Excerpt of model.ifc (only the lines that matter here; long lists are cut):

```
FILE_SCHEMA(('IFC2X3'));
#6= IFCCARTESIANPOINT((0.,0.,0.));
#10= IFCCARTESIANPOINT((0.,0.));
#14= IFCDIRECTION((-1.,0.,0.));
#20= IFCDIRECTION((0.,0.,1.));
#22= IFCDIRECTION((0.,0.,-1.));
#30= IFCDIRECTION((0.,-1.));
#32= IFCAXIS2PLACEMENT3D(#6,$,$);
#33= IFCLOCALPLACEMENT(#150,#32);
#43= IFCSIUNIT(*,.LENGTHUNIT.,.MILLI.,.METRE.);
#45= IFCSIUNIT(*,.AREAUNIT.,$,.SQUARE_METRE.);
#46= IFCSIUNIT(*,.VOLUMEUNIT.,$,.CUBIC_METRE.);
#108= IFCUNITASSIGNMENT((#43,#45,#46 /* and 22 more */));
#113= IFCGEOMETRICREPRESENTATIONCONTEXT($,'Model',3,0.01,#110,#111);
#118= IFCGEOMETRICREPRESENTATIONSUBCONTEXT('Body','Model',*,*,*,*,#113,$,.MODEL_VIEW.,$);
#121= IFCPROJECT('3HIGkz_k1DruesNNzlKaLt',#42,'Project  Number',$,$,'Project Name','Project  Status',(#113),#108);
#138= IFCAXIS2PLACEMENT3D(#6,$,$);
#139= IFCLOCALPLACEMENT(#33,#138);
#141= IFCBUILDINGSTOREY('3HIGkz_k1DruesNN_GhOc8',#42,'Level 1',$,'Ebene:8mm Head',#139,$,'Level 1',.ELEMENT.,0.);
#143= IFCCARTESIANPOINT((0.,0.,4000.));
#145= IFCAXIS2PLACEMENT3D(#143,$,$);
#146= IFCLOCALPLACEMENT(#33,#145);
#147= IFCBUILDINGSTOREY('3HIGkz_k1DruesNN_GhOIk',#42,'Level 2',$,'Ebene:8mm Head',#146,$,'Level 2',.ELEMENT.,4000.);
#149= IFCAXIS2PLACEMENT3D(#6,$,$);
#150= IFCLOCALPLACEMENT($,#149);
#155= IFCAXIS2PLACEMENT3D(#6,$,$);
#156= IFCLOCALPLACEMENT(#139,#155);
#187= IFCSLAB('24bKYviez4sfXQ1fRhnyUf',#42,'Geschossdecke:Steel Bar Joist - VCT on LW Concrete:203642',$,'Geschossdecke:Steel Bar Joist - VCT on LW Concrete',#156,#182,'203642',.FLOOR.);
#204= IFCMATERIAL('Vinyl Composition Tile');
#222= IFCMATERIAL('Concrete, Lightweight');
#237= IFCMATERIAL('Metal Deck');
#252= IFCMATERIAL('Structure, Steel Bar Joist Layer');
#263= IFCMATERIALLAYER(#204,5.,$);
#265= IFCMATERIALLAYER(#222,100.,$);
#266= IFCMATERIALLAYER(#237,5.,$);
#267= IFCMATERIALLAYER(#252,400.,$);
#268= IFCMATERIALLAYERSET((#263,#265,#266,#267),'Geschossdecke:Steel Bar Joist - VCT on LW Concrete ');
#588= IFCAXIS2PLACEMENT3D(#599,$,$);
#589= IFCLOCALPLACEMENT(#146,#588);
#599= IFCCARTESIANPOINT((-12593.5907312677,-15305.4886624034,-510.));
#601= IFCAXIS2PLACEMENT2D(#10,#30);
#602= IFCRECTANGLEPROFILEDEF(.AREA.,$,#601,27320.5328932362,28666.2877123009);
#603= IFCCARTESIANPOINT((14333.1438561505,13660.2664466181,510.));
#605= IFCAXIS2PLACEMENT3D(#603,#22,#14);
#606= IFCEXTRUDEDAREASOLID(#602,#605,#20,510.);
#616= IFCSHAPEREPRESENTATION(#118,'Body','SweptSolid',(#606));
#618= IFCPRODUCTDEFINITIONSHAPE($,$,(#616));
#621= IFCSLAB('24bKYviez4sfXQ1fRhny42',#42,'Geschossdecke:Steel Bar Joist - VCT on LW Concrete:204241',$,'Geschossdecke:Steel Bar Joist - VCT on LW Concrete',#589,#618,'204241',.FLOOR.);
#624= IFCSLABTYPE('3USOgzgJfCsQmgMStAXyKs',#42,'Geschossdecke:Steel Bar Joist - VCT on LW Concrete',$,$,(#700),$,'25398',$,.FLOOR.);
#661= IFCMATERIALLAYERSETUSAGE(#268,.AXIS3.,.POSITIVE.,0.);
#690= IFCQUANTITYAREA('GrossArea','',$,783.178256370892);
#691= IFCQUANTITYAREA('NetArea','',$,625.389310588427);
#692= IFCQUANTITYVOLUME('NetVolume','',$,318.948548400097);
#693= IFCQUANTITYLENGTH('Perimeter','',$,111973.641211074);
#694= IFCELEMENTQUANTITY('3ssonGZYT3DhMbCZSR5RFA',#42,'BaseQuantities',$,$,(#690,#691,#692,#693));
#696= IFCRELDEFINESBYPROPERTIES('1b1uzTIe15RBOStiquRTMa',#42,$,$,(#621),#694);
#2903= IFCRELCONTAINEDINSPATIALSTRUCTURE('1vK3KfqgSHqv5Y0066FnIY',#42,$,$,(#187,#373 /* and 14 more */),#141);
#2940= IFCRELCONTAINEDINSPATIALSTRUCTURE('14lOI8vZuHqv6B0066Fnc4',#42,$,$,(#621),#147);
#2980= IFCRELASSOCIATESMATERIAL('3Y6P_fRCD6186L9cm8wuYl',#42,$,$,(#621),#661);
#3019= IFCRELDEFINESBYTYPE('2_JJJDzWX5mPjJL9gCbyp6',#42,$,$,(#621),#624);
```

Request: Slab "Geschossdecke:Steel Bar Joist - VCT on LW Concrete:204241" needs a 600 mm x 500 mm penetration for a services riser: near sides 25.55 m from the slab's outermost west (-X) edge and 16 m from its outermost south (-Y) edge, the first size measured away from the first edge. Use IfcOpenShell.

```python
import numpy as np
import ifcopenshell
import ifcopenshell.api.feature
import ifcopenshell.api.geometry
import ifcopenshell.api.pset
import ifcopenshell.api.root
import ifcopenshell.geom
import ifcopenshell.util.element
import ifcopenshell.util.placement
import ifcopenshell.util.representation
import ifcopenshell.util.shape
import ifcopenshell.util.unit

model = ifcopenshell.open("model.ifc")
unit_scale = ifcopenshell.util.unit.calculate_unit_scale(model)
area_scale = ifcopenshell.util.unit.calculate_unit_scale(model, "AREAUNIT")
volume_scale = ifcopenshell.util.unit.calculate_unit_scale(model, "VOLUMEUNIT")
settings = ifcopenshell.geom.settings()


def volume(element):
    """Net volume in cubic metres, openings subtracted."""
    shape = ifcopenshell.geom.create_shape(settings, element)
    return ifcopenshell.util.shape.get_volume(shape.geometry)


slab = model.by_id(621)
before = volume(slab)

# Extent in the slab's own axes, in metres. The edges named are its -X and -Y sides.
slab_shape = ifcopenshell.geom.create_shape(settings, slab)
vertices = ifcopenshell.util.shape.get_vertices(slab_shape.geometry)
x_min, y_min, bottom = vertices.min(axis=0)
top = vertices[:, 2].max()

opening = ifcopenshell.api.root.create_entity(model, ifc_class="IfcOpeningElement", name="Services riser opening")
context = ifcopenshell.util.representation.get_context(model, "Model", "Body", "MODEL_VIEW")
width, depth = 0.6, 0.5
outline = [(0.0, 0.0), (width, 0.0), (width, depth), (0.0, depth), (0.0, 0.0)]
# Overshoot both faces by 50 mm so the cut is clean.
shape = ifcopenshell.api.geometry.add_slab_representation(
    model, context=context, depth=top - bottom + 0.1, polyline=outline
)
ifcopenshell.api.geometry.assign_representation(model, product=opening, representation=shape)

matrix = ifcopenshell.util.placement.get_local_placement(slab.ObjectPlacement)
matrix[:, 3] = matrix @ np.append(np.array([x_min + 25.55, y_min + 16, bottom - 0.05]) / unit_scale, 1.0)
ifcopenshell.api.geometry.edit_object_placement(model, product=opening, matrix=matrix, is_si=False)
ifcopenshell.api.feature.add_feature(model, feature=opening, element=slab)

after = volume(slab)

# Update the slab's stored quantities.
qto = model.by_id(ifcopenshell.util.element.get_pset(slab, "BaseQuantities", should_inherit=False)["id"])
ifcopenshell.api.pset.edit_qto(model, qto=qto, properties={
    "NetArea": after / (top - bottom) / area_scale,
    "NetVolume": after / volume_scale,
})

print(f"slab volume {before:.3f} -> {after:.3f} m3")

model.write("model_updated.ifc")
```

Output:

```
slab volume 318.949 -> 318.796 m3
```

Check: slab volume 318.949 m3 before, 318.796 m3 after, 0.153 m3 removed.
